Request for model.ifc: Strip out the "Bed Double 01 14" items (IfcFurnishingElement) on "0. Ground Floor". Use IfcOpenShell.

First a look at what the model holds.

```python
import ifcopenshell
import ifcopenshell.util.element

model = ifcopenshell.open("model.ifc")
print(model.schema)
storey = next(s for s in model.by_type("IfcBuildingStorey") if s.Name == "0. Ground Floor")
furniture = [e for e in ifcopenshell.util.element.get_decomposition(storey) if e.is_a("IfcFurnishingElement")]
seen = {}
for e in furniture:
    element_type = ifcopenshell.util.element.get_type(e)
    name = element_type.Name if element_type not in (None, e) else None
    seen[name] = seen.get(name, 0) + 1
for name, count in sorted(seen.items(), key=str):
    print(count, "x", name)
```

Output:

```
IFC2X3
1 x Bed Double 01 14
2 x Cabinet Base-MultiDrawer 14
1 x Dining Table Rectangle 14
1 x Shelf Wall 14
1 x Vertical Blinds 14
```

```python
import ifcopenshell
import ifcopenshell.api.root
import ifcopenshell.util.element

model = ifcopenshell.open("model.ifc")

storey = next(s for s in model.by_type("IfcBuildingStorey") if s.Name == "0. Ground Floor")
furniture = [e for e in ifcopenshell.util.element.get_decomposition(storey) if e.is_a("IfcFurnishingElement")]
targets = [e for e in furniture if (t := ifcopenshell.util.element.get_type(e)) not in (None, e) and t.Name == "Bed Double 01 14"]

for e in targets:
    ifcopenshell.api.root.remove_product(model, product=e)
print(len(targets), "removed")

model.write("model_v2.ifc")
```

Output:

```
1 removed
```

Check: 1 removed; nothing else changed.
